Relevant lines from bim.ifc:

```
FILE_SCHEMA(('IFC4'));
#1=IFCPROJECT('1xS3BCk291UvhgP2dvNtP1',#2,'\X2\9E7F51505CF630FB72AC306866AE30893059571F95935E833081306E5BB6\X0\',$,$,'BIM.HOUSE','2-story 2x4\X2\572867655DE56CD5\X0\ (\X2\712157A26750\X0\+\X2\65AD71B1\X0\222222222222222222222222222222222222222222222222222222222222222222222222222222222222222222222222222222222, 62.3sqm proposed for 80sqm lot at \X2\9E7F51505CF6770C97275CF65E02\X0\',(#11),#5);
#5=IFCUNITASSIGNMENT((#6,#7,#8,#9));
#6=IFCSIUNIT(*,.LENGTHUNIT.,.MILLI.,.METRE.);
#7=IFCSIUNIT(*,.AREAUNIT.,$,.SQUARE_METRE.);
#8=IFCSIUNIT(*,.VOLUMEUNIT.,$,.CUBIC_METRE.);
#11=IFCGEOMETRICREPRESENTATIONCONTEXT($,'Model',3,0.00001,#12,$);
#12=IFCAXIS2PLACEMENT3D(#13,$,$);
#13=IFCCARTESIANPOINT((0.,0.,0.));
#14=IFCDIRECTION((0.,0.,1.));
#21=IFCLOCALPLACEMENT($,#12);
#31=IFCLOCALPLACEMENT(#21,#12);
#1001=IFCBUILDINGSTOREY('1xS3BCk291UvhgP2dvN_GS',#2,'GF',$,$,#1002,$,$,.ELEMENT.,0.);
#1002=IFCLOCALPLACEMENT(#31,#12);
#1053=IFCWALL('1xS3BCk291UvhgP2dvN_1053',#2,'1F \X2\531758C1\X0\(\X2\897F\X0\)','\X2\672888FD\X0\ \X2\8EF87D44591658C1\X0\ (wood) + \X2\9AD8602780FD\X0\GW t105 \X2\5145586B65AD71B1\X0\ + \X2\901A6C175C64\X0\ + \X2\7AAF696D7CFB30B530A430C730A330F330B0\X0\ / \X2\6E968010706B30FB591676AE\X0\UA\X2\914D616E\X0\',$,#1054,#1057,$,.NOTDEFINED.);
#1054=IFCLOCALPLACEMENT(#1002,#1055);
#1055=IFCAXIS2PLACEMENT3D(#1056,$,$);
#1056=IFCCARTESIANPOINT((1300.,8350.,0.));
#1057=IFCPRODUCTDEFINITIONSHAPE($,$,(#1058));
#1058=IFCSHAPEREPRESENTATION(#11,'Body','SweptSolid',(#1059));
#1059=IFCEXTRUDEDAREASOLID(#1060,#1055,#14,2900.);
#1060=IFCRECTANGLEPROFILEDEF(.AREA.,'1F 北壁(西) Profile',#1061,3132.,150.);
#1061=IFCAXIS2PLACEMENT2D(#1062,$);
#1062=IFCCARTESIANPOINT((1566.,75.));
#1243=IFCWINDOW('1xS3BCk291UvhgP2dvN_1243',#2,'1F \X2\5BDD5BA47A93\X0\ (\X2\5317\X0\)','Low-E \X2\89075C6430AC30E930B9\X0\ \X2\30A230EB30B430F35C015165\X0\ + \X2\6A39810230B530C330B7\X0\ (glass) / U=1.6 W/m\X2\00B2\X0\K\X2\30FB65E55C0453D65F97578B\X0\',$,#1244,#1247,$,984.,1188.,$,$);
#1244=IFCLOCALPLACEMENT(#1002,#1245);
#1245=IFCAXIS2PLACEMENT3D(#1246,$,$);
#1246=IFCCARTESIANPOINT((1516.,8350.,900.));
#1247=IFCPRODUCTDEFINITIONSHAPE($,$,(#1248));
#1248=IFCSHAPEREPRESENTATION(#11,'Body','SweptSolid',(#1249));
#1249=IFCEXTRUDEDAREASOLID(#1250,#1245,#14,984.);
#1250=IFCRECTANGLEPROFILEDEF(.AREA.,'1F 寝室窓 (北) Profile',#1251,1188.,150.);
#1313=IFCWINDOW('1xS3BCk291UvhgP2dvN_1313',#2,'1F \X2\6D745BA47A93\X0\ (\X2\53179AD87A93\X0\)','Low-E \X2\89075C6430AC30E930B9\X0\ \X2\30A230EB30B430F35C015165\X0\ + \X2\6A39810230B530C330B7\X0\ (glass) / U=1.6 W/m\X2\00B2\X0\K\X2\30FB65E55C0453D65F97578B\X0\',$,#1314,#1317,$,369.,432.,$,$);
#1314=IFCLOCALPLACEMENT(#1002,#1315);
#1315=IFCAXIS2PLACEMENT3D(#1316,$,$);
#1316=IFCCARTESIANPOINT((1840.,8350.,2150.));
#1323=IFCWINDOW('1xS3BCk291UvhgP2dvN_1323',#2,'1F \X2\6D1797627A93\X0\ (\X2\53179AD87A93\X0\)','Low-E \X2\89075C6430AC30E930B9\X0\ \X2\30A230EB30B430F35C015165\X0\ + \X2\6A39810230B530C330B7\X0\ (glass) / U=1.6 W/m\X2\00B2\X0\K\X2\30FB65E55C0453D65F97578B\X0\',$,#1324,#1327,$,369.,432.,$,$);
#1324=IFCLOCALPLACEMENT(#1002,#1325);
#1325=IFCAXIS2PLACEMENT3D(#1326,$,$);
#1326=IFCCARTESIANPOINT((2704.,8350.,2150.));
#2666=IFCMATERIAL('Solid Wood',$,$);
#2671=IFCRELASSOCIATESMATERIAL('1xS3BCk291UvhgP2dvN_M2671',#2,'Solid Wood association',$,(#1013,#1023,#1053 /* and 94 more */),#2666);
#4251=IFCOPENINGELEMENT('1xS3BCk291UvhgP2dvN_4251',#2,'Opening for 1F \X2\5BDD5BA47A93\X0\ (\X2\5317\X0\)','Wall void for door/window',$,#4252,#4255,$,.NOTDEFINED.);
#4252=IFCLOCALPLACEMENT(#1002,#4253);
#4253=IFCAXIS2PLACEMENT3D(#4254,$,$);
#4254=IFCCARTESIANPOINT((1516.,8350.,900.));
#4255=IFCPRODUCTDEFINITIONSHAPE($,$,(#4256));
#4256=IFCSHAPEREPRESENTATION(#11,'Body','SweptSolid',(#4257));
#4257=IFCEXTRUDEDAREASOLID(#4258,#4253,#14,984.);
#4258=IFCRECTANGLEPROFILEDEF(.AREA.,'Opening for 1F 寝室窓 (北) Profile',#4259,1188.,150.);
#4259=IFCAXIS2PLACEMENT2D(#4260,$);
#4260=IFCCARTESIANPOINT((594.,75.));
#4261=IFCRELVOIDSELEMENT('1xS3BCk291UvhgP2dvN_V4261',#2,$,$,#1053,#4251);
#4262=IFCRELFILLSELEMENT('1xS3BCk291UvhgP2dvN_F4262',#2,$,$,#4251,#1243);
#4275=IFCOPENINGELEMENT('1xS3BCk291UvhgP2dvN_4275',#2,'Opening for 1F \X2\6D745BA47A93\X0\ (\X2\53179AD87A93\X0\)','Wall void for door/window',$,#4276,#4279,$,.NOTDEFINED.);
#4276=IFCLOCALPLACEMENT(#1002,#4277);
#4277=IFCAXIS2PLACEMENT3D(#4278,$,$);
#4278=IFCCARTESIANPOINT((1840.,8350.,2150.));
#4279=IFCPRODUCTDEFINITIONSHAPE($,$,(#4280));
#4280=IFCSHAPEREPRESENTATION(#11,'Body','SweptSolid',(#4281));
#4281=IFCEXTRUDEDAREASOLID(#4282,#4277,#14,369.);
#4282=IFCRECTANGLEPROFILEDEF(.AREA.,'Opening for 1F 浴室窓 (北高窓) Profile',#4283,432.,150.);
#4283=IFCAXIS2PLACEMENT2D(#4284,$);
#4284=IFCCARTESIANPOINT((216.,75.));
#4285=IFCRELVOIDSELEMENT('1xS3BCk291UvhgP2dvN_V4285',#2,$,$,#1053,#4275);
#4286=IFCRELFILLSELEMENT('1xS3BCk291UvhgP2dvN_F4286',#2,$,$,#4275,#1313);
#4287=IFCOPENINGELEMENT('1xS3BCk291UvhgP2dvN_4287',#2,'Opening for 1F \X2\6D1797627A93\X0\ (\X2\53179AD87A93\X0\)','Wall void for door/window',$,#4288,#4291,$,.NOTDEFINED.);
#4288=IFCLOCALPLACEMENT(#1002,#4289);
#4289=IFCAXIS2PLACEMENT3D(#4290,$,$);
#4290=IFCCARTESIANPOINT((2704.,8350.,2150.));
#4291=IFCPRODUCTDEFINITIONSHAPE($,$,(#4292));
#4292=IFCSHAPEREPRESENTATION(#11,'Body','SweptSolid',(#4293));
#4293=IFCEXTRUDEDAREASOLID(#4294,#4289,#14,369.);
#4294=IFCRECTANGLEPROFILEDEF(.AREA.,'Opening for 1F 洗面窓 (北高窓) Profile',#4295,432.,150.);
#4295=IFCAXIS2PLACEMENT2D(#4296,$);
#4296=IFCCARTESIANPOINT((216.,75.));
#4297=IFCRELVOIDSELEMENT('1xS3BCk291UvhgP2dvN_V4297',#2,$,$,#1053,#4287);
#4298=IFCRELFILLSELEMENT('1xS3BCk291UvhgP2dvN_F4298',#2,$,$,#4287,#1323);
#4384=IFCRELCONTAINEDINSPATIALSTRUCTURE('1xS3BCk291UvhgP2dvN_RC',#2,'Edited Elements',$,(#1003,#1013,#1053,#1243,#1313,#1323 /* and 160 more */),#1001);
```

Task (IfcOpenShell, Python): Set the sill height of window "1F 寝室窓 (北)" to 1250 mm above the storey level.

```python
import numpy as np
import ifcopenshell
import ifcopenshell.api.geometry
import ifcopenshell.geom
import ifcopenshell.util.element
import ifcopenshell.util.placement
import ifcopenshell.util.shape
import ifcopenshell.util.unit

model = ifcopenshell.open("bim.ifc")
unit_scale = ifcopenshell.util.unit.calculate_unit_scale(model)

window = model.by_guid("1xS3BCk291UvhgP2dvN_1243")
opening = window.FillsVoids[0].RelatingOpeningElement
storey = ifcopenshell.util.element.get_container(window, ifc_class="IfcBuildingStorey")
level = ifcopenshell.util.placement.get_local_placement(storey.ObjectPlacement)[2, 3]

# The opening's origin need not be at the sill, so measure its lowest point.
shape = ifcopenshell.geom.create_shape(ifcopenshell.geom.settings(), opening)
bottom = ifcopenshell.util.shape.get_shape_bottom_elevation(shape, shape.geometry) / unit_scale
dz = level + 1250.0 - bottom

shift = np.array([0.0, 0.0, dz])
# The window is not placed relative to its opening, so move both.
for product in (opening, window):
    matrix = ifcopenshell.util.placement.get_local_placement(product.ObjectPlacement)
    matrix[:3, 3] += shift
    ifcopenshell.api.geometry.edit_object_placement(model, product=product, matrix=matrix, is_si=False)

print(f"moved by {dz * unit_scale:+.3f} m")

model.write("bim_updated.ifc")
```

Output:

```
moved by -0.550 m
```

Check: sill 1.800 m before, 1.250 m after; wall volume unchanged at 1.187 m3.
